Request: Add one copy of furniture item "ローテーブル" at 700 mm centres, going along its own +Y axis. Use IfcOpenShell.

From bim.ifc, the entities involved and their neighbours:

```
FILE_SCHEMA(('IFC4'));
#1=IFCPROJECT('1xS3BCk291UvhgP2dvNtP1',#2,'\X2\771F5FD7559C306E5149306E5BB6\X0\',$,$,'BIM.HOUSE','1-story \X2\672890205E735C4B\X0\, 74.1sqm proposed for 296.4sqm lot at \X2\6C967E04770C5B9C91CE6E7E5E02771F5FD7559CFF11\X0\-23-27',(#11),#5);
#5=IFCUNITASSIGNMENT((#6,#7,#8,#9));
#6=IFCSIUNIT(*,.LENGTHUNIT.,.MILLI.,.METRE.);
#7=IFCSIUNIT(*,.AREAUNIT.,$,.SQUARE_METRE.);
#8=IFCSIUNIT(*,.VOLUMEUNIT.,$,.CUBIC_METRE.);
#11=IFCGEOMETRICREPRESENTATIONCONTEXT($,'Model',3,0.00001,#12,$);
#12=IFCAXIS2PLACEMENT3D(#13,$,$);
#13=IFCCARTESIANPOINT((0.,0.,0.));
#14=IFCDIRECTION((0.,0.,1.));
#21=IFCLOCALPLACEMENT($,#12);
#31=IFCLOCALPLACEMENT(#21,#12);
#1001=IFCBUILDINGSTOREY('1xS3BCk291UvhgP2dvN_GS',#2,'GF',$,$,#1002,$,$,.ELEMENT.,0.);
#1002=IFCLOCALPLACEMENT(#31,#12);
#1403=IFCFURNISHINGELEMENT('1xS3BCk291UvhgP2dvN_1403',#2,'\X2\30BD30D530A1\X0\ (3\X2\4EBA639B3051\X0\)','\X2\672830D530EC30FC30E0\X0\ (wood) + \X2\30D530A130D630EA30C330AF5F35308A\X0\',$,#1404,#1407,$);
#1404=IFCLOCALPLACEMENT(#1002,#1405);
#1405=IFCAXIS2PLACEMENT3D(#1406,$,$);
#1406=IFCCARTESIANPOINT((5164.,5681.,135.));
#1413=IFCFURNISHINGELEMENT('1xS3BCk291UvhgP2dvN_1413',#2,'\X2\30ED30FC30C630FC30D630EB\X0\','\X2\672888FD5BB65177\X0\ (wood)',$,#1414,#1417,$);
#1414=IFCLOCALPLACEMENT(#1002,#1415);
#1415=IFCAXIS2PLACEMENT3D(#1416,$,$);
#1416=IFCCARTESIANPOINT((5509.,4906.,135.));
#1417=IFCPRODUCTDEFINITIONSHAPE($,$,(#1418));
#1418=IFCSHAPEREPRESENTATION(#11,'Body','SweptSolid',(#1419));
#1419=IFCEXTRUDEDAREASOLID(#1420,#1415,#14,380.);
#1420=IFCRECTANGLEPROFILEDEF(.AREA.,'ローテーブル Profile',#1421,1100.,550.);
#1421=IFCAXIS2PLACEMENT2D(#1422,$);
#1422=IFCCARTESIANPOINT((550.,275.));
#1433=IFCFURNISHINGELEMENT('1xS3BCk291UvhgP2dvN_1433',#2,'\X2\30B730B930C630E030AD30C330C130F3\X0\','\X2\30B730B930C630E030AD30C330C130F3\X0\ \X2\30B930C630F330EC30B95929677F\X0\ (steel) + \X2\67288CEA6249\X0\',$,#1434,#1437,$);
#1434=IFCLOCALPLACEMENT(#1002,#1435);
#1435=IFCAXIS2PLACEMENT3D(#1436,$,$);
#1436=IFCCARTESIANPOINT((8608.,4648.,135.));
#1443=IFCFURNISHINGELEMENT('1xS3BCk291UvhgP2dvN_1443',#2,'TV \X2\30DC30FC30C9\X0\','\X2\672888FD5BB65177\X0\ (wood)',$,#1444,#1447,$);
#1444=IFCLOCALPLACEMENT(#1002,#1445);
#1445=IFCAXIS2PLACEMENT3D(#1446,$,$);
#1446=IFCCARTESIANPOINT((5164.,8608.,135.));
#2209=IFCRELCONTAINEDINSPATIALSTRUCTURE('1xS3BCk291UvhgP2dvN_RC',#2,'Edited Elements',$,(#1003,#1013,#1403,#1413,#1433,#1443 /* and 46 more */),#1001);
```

```python
import ifcopenshell
import ifcopenshell.api.geometry
import ifcopenshell.api.root
import ifcopenshell.util.element
import ifcopenshell.util.placement

model = ifcopenshell.open("bim.ifc")


def reuse_history(source, copy):
    """copy_class also copies each property set's owner history, people and application; keep the originals."""
    for rel in copy.IsDefinedBy:
        if rel.is_a("IfcRelDefinesByProperties") and (history := rel.RelatingPropertyDefinition.OwnerHistory):
            rel.RelatingPropertyDefinition.OwnerHistory = source.OwnerHistory
            ifcopenshell.util.element.remove_deep2(model, history)


source = model.by_id(1413)
base = ifcopenshell.util.placement.get_local_placement(source.ObjectPlacement)
step = base[:3, 1] * 700.0

for i in range(1, 2):
    copy = ifcopenshell.api.root.copy_class(model, product=source)
    copy.Representation = ifcopenshell.util.element.copy_deep(
        model, source.Representation, exclude=["IfcGeometricRepresentationContext", "IfcRepresentationMap"]
    )
    reuse_history(source, copy)
    matrix = base.copy()
    matrix[:3, 3] += i * step
    print("added at", matrix[:3, 3].round(3) + 0.0)
    ifcopenshell.api.geometry.edit_object_placement(model, product=copy, matrix=matrix, is_si=False)

model.write("bim_rev.ifc")
```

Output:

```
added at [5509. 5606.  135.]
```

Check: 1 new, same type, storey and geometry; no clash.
